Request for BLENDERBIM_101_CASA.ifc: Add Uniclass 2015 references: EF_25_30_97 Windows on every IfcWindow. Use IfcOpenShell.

First a look at what the model holds.

```python
import ifcopenshell

model = ifcopenshell.open("BLENDERBIM_101_CASA.ifc")
print(model.schema)
print("classifications:", [c.Name for c in model.by_type("IfcClassification")])
for ifc_class in ("IfcDoor", "IfcRoof", "IfcStair", "IfcWall", "IfcWindow"):
    print(ifc_class, len(model.by_type(ifc_class)))
```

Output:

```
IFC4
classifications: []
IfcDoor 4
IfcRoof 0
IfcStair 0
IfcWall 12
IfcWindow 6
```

```python
import ifcopenshell
import ifcopenshell.api.classification

model = ifcopenshell.open("BLENDERBIM_101_CASA.ifc")

system = ifcopenshell.api.classification.add_classification(model, classification="Uniclass 2015")

codes = {
    "IfcWindow": ("EF_25_30_97", "Windows"),
}
for ifc_class, (code, name) in codes.items():
    products = model.by_type(ifc_class)
    ifcopenshell.api.classification.add_reference(
        model, products=products, classification=system, identification=code, name=name
    )
    print(code, len(products))

model.write("BLENDERBIM_101_CASA_edited.ifc")
```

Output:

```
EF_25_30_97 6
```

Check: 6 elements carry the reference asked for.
